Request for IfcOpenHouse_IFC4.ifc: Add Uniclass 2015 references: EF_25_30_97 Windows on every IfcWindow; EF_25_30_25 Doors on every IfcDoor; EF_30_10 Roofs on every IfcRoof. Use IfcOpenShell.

First a look at what the model holds.

```python
import ifcopenshell

model = ifcopenshell.open("IfcOpenHouse_IFC4.ifc")
print(model.schema)
print("classifications:", [c.Name for c in model.by_type("IfcClassification")])
for ifc_class in ("IfcDoor", "IfcRoof", "IfcStair", "IfcWall", "IfcWindow"):
    print(ifc_class, len(model.by_type(ifc_class)))
```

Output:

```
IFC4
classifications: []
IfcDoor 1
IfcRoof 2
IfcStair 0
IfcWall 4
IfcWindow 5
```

```python
import ifcopenshell
import ifcopenshell.api.classification

model = ifcopenshell.open("IfcOpenHouse_IFC4.ifc")

system = ifcopenshell.api.classification.add_classification(model, classification="Uniclass 2015")

codes = {
    "IfcWindow": ("EF_25_30_97", "Windows"),
    "IfcDoor": ("EF_25_30_25", "Doors"),
    "IfcRoof": ("EF_30_10", "Roofs"),
}
for ifc_class, (code, name) in codes.items():
    products = model.by_type(ifc_class)
    ifcopenshell.api.classification.add_reference(
        model, products=products, classification=system, identification=code, name=name
    )
    print(code, len(products))

model.write("IfcOpenHouse_IFC4_updated.ifc")
```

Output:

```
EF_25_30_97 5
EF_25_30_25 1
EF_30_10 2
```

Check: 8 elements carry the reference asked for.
